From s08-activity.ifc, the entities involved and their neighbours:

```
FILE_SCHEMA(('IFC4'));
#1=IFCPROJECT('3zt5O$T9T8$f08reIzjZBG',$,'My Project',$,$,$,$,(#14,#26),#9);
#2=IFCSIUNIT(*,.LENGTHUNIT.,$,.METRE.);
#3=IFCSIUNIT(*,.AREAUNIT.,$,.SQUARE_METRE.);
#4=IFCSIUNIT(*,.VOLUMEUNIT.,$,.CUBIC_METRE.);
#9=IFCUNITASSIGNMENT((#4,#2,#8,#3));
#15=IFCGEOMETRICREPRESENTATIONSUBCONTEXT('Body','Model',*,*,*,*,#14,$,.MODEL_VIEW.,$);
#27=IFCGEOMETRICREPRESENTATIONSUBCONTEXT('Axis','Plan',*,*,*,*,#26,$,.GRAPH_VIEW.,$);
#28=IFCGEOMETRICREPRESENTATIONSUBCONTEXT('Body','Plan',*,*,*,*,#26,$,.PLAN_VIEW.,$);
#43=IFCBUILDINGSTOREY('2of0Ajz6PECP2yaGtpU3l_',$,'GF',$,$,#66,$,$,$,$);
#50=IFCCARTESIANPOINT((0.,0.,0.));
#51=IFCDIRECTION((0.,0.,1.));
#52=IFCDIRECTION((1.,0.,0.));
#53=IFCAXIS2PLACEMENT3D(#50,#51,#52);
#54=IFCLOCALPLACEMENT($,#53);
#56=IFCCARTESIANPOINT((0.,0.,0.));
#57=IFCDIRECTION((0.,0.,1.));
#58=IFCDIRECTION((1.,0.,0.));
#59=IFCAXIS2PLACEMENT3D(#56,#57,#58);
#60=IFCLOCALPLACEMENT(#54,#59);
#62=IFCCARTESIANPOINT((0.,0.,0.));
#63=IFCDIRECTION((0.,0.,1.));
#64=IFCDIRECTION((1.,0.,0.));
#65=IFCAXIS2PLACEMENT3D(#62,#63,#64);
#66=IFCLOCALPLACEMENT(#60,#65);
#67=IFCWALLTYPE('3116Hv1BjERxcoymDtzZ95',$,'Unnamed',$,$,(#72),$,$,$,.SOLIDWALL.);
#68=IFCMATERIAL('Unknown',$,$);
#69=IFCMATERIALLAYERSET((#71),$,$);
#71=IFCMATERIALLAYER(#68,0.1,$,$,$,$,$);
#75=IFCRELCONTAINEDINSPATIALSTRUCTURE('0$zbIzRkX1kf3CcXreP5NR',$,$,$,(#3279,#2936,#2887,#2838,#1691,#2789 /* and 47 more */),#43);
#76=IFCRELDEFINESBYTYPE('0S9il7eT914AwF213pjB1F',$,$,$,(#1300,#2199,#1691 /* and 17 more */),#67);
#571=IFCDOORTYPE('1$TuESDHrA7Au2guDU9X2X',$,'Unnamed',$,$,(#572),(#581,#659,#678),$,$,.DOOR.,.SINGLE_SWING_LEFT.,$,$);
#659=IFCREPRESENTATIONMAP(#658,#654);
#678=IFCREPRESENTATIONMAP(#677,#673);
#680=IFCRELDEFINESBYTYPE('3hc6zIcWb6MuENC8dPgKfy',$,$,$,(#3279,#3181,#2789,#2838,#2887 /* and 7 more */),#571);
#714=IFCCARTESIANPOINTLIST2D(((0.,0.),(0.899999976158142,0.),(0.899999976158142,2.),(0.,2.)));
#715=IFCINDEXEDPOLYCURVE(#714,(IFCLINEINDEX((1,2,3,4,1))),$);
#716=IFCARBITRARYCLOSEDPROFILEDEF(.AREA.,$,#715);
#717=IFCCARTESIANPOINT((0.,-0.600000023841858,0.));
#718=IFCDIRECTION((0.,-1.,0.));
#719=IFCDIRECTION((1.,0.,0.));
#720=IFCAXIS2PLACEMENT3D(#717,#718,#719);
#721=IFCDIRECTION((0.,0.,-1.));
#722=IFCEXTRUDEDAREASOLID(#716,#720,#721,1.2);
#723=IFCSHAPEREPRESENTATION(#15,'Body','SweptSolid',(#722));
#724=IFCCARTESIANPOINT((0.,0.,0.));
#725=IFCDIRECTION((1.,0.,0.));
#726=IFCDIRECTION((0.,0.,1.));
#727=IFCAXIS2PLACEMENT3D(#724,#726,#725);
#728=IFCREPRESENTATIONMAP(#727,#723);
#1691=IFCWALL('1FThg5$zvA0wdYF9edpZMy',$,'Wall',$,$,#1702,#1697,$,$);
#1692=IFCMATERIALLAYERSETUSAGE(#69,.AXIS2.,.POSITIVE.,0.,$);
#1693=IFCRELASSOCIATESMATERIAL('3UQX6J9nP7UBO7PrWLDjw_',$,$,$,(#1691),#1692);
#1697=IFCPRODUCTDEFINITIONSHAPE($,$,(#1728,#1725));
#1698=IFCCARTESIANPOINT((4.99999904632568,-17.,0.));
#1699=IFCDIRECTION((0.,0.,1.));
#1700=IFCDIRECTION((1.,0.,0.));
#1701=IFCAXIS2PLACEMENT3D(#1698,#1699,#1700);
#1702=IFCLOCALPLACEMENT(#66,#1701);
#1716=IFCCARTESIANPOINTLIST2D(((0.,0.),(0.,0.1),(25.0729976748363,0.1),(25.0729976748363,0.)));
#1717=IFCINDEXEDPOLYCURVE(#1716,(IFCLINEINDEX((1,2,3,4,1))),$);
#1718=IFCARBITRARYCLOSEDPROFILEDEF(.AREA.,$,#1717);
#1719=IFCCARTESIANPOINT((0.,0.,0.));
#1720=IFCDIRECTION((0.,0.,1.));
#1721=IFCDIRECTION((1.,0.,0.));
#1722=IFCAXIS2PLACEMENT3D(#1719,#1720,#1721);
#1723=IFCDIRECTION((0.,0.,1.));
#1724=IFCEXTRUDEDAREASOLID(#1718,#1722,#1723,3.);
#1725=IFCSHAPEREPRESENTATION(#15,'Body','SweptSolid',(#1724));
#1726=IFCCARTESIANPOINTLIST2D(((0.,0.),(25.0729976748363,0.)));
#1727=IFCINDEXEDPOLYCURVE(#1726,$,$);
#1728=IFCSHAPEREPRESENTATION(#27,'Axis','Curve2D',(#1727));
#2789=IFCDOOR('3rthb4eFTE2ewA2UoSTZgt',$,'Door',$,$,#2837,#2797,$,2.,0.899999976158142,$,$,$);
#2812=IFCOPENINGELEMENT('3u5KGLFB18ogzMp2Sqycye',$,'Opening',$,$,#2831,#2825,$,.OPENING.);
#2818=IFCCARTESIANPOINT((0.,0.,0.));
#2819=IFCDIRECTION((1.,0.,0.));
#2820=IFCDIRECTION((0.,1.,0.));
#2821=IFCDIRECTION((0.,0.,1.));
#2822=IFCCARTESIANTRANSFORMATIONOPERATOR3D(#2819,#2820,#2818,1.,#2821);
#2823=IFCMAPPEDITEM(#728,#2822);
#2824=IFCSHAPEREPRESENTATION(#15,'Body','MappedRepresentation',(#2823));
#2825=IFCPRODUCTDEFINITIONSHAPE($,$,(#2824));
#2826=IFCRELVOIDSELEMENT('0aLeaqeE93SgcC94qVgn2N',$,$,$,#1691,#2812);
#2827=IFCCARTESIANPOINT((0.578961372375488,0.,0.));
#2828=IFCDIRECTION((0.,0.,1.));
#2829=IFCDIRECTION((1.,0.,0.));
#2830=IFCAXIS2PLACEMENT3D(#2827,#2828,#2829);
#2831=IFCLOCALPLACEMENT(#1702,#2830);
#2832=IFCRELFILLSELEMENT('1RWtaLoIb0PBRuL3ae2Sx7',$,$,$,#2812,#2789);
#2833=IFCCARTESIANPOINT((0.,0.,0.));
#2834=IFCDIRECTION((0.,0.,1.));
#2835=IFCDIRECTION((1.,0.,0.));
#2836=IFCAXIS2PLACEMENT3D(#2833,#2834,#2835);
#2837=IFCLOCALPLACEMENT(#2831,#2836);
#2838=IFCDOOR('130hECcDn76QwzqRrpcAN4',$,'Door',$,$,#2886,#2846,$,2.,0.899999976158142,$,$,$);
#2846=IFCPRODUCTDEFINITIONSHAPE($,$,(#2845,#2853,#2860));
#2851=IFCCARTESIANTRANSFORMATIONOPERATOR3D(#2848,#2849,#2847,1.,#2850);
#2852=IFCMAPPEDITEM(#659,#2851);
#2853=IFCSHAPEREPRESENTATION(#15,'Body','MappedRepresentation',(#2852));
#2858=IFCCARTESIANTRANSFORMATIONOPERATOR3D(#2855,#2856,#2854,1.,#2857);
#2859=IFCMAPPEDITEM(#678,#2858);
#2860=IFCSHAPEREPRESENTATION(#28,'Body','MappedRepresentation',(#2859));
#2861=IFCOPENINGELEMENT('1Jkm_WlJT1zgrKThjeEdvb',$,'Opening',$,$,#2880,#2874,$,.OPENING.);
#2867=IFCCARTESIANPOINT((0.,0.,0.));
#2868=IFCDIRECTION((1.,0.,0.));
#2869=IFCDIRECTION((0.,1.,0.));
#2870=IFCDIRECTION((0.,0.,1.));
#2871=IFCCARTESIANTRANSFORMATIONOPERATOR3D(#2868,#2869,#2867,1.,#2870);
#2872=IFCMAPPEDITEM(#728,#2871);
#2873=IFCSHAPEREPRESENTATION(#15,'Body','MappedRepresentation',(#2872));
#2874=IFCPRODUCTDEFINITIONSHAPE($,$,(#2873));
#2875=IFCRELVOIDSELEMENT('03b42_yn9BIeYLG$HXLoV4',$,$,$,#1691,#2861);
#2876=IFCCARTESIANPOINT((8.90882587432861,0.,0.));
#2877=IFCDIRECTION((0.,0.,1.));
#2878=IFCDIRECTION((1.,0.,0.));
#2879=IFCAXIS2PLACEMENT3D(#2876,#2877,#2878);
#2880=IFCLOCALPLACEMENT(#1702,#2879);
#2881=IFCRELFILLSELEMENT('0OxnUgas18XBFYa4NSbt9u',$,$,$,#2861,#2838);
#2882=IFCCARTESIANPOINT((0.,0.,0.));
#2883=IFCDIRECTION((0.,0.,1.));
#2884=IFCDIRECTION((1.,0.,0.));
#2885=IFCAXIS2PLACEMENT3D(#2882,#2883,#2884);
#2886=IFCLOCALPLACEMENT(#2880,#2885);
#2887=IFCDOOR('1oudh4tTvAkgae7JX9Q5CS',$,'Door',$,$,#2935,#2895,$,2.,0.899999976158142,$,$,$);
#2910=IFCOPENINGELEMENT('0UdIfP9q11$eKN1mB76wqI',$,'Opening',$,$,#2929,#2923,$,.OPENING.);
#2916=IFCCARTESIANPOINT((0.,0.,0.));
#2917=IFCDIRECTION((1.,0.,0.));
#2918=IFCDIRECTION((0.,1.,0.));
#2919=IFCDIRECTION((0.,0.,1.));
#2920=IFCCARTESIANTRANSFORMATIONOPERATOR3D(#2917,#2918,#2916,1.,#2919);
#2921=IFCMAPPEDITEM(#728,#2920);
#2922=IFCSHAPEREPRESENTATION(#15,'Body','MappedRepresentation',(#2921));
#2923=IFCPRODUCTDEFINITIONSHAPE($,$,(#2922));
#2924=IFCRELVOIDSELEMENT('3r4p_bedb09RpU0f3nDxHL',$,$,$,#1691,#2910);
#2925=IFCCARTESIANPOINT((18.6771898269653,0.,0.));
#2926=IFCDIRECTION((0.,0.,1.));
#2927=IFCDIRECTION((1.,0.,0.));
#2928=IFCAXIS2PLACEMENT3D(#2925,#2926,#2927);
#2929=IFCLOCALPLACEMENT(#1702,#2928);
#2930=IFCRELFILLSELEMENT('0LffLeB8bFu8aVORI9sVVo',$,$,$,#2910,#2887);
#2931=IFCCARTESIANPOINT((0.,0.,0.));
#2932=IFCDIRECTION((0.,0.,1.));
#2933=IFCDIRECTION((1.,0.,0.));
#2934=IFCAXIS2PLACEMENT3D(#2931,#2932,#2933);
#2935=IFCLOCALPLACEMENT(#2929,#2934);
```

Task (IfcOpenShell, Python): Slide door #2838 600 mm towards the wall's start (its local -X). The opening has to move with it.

```python
import ifcopenshell
import ifcopenshell.api.geometry
import ifcopenshell.util.placement
import ifcopenshell.util.unit

model = ifcopenshell.open("s08-activity.ifc")
unit_scale = ifcopenshell.util.unit.calculate_unit_scale(model)

door = model.by_guid("130hECcDn76QwzqRrpcAN4")
opening = door.FillsVoids[0].RelatingOpeningElement
wall = opening.VoidsElements[0].RelatingBuildingElement

wall_matrix = ifcopenshell.util.placement.get_local_placement(wall.ObjectPlacement)
shift = wall_matrix[:3, 0] * -0.6 / unit_scale
before = ifcopenshell.util.placement.get_local_placement(door.ObjectPlacement)[:3, 3].copy()

# The door is placed relative to its opening, so it follows when the opening moves.
matrix = ifcopenshell.util.placement.get_local_placement(opening.ObjectPlacement)
matrix[:3, 3] += shift
ifcopenshell.api.geometry.edit_object_placement(
    model, product=opening, matrix=matrix, is_si=False, should_transform_children=True
)

after = ifcopenshell.util.placement.get_local_placement(door.ObjectPlacement)[:3, 3]
print("door moved by", (after - before).round(3) + 0.0)

model.write("s08-activity_updated.ifc")
```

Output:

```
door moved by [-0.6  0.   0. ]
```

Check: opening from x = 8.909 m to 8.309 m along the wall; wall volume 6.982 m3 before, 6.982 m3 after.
